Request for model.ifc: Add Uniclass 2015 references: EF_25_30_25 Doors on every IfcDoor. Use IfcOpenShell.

First a look at what the model holds.

```python
import ifcopenshell

model = ifcopenshell.open("model.ifc")
print(model.schema)
print("classifications:", [c.Name for c in model.by_type("IfcClassification")])
for ifc_class in ("IfcDoor", "IfcRoof", "IfcStair", "IfcWall", "IfcWindow"):
    print(ifc_class, len(model.by_type(ifc_class)))
```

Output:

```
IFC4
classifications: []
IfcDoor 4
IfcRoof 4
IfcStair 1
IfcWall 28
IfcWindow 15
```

```python
import ifcopenshell
import ifcopenshell.api.classification

model = ifcopenshell.open("model.ifc")

system = ifcopenshell.api.classification.add_classification(model, classification="Uniclass 2015")

codes = {
    "IfcDoor": ("EF_25_30_25", "Doors"),
}
for ifc_class, (code, name) in codes.items():
    products = model.by_type(ifc_class)
    ifcopenshell.api.classification.add_reference(
        model, products=products, classification=system, identification=code, name=name
    )
    print(code, len(products))

model.write("model-out.ifc")
```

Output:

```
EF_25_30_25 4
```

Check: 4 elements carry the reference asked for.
